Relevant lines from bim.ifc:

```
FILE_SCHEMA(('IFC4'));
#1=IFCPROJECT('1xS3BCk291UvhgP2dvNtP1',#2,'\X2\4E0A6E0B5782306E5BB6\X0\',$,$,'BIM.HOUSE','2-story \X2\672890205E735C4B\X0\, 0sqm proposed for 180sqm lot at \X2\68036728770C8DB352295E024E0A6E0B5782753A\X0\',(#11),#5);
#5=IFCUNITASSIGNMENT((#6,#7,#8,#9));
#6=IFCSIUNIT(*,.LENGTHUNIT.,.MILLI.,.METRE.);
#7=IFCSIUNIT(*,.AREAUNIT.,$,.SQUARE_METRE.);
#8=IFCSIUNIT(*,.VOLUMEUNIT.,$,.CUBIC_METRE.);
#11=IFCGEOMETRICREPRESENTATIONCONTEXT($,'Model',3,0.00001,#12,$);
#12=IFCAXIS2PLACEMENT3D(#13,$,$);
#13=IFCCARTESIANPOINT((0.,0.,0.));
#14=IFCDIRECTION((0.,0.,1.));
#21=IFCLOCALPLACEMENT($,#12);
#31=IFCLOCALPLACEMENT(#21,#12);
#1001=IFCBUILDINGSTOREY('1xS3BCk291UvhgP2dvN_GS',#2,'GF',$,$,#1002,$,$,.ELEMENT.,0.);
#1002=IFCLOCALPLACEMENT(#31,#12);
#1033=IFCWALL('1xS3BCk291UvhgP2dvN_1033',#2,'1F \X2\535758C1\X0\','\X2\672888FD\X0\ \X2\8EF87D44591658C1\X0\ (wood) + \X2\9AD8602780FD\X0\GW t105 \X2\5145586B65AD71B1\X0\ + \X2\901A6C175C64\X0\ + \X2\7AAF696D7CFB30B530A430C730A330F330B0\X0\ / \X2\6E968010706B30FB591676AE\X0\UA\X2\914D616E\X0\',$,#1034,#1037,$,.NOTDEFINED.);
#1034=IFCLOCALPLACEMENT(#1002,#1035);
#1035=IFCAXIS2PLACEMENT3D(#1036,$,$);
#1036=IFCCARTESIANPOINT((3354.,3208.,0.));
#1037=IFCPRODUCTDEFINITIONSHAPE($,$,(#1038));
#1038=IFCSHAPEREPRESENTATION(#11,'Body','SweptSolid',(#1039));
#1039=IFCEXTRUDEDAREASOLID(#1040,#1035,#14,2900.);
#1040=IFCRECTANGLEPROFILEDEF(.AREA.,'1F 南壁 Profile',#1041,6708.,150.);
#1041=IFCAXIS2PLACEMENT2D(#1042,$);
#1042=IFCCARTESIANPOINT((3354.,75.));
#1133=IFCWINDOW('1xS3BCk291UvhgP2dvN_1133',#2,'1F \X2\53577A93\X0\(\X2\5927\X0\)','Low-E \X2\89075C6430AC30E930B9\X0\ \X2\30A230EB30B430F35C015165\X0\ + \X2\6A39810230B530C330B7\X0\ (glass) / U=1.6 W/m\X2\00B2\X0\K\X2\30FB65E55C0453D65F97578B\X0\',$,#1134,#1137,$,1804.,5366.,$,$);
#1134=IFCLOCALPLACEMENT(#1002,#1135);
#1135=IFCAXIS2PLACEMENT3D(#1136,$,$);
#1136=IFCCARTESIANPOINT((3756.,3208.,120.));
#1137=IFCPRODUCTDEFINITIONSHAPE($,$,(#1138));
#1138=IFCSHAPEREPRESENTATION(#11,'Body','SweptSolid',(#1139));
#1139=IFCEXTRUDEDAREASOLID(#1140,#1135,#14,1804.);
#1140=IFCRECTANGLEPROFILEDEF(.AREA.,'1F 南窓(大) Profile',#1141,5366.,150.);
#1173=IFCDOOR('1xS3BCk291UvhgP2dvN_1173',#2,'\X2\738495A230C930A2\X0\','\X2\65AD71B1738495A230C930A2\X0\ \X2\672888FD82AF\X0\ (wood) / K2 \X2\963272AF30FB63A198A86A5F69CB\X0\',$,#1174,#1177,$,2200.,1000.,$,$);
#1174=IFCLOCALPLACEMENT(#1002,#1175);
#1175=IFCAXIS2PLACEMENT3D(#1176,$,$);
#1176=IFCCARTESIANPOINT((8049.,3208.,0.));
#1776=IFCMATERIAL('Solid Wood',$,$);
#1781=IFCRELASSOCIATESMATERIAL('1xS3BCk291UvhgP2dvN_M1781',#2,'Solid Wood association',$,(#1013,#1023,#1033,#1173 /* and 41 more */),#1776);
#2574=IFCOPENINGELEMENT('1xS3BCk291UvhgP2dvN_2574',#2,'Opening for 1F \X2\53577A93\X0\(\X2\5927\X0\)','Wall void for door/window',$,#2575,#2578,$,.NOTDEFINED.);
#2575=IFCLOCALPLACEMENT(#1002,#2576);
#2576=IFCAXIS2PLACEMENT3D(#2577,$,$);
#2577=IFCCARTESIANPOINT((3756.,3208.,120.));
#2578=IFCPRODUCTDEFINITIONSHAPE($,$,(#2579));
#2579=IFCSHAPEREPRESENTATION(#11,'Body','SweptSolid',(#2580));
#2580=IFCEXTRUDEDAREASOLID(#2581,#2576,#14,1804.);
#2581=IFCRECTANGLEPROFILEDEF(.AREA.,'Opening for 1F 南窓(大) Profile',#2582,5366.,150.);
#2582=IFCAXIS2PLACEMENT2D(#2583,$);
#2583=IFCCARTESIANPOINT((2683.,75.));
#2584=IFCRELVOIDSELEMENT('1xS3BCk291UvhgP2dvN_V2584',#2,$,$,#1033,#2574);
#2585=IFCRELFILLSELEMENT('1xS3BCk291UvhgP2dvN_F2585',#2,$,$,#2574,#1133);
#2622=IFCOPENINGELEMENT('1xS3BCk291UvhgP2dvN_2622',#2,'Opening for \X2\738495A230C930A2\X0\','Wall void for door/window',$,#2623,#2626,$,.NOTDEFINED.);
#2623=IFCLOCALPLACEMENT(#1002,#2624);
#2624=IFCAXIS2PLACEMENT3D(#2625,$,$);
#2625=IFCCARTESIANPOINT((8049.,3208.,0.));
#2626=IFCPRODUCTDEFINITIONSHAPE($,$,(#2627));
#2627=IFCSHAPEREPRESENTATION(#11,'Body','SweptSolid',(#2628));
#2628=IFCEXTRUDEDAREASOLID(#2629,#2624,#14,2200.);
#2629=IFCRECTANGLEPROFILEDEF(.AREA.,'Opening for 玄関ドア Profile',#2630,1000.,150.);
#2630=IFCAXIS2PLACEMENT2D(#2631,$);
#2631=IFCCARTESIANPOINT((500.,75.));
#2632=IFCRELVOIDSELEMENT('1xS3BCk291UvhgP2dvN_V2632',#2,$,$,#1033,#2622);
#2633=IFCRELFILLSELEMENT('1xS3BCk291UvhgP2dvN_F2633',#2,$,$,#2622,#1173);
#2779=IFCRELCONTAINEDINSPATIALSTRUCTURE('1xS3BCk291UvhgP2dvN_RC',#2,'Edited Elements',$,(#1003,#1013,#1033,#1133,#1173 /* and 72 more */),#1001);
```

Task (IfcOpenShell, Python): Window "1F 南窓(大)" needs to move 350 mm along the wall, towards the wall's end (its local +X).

```python
import ifcopenshell
import ifcopenshell.api.geometry
import ifcopenshell.util.placement
import ifcopenshell.util.unit

model = ifcopenshell.open("bim.ifc")
unit_scale = ifcopenshell.util.unit.calculate_unit_scale(model)

window = model.by_guid("1xS3BCk291UvhgP2dvN_1133")
opening = window.FillsVoids[0].RelatingOpeningElement
wall = opening.VoidsElements[0].RelatingBuildingElement

wall_matrix = ifcopenshell.util.placement.get_local_placement(wall.ObjectPlacement)
shift = wall_matrix[:3, 0] * 0.35 / unit_scale
before = ifcopenshell.util.placement.get_local_placement(window.ObjectPlacement)[:3, 3].copy()

# The window is not placed relative to its opening, so move both.
for product in (opening, window):
    matrix = ifcopenshell.util.placement.get_local_placement(product.ObjectPlacement)
    matrix[:3, 3] += shift
    ifcopenshell.api.geometry.edit_object_placement(model, product=product, matrix=matrix, is_si=False)

after = ifcopenshell.util.placement.get_local_placement(window.ObjectPlacement)[:3, 3]
print("window moved by", (after - before).round(3) + 0.0)

model.write("bim-out.ifc")
```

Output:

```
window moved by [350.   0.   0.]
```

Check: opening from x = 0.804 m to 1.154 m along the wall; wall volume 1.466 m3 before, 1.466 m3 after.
